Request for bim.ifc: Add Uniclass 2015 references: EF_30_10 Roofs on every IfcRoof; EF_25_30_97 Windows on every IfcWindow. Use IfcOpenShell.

First a look at what the model holds.

```python
import ifcopenshell

model = ifcopenshell.open("bim.ifc")
print(model.schema)
print("classifications:", [c.Name for c in model.by_type("IfcClassification")])
for ifc_class in ("IfcDoor", "IfcRoof", "IfcStair", "IfcWall", "IfcWindow"):
    print(ifc_class, len(model.by_type(ifc_class)))
```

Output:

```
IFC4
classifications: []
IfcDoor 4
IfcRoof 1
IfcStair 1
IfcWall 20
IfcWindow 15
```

```python
import ifcopenshell
import ifcopenshell.api.classification

model = ifcopenshell.open("bim.ifc")

system = ifcopenshell.api.classification.add_classification(model, classification="Uniclass 2015")

codes = {
    "IfcRoof": ("EF_30_10", "Roofs"),
    "IfcWindow": ("EF_25_30_97", "Windows"),
}
for ifc_class, (code, name) in codes.items():
    products = model.by_type(ifc_class)
    ifcopenshell.api.classification.add_reference(
        model, products=products, classification=system, identification=code, name=name
    )
    print(code, len(products))

model.write("bim-out.ifc")
```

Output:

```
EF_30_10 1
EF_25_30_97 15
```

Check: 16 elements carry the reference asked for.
